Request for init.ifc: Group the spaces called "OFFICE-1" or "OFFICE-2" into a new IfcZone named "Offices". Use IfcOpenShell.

First a look at what the model holds.

```python
import ifcopenshell

model = ifcopenshell.open("init.ifc")
print(model.schema)
seen = {}
for space in model.by_type("IfcSpace"):
    seen[space.Name] = seen.get(space.Name, 0) + 1
for name, count in sorted(seen.items(), key=str):
    print(count, "x", name)
print("zones:", [z.Name for z in model.by_type("IfcZone")][:20])
```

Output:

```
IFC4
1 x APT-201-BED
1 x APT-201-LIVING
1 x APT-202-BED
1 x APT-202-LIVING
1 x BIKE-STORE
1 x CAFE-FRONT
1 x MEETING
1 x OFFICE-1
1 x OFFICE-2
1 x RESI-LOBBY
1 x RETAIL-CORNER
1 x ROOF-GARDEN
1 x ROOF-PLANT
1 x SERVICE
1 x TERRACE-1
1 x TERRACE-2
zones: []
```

```python
import ifcopenshell
import ifcopenshell.api.group
import ifcopenshell.api.root

model = ifcopenshell.open("init.ifc")

names = {"OFFICE-1", "OFFICE-2"}
spaces = [s for s in model.by_type("IfcSpace") if s.Name in names]

zone = ifcopenshell.api.root.create_entity(model, ifc_class="IfcZone", name="Offices")
ifcopenshell.api.group.assign_group(model, products=spaces, group=zone)
print(len(spaces), "spaces in", zone.Name)

model.write("init-out.ifc")
```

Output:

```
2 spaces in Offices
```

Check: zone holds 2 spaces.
